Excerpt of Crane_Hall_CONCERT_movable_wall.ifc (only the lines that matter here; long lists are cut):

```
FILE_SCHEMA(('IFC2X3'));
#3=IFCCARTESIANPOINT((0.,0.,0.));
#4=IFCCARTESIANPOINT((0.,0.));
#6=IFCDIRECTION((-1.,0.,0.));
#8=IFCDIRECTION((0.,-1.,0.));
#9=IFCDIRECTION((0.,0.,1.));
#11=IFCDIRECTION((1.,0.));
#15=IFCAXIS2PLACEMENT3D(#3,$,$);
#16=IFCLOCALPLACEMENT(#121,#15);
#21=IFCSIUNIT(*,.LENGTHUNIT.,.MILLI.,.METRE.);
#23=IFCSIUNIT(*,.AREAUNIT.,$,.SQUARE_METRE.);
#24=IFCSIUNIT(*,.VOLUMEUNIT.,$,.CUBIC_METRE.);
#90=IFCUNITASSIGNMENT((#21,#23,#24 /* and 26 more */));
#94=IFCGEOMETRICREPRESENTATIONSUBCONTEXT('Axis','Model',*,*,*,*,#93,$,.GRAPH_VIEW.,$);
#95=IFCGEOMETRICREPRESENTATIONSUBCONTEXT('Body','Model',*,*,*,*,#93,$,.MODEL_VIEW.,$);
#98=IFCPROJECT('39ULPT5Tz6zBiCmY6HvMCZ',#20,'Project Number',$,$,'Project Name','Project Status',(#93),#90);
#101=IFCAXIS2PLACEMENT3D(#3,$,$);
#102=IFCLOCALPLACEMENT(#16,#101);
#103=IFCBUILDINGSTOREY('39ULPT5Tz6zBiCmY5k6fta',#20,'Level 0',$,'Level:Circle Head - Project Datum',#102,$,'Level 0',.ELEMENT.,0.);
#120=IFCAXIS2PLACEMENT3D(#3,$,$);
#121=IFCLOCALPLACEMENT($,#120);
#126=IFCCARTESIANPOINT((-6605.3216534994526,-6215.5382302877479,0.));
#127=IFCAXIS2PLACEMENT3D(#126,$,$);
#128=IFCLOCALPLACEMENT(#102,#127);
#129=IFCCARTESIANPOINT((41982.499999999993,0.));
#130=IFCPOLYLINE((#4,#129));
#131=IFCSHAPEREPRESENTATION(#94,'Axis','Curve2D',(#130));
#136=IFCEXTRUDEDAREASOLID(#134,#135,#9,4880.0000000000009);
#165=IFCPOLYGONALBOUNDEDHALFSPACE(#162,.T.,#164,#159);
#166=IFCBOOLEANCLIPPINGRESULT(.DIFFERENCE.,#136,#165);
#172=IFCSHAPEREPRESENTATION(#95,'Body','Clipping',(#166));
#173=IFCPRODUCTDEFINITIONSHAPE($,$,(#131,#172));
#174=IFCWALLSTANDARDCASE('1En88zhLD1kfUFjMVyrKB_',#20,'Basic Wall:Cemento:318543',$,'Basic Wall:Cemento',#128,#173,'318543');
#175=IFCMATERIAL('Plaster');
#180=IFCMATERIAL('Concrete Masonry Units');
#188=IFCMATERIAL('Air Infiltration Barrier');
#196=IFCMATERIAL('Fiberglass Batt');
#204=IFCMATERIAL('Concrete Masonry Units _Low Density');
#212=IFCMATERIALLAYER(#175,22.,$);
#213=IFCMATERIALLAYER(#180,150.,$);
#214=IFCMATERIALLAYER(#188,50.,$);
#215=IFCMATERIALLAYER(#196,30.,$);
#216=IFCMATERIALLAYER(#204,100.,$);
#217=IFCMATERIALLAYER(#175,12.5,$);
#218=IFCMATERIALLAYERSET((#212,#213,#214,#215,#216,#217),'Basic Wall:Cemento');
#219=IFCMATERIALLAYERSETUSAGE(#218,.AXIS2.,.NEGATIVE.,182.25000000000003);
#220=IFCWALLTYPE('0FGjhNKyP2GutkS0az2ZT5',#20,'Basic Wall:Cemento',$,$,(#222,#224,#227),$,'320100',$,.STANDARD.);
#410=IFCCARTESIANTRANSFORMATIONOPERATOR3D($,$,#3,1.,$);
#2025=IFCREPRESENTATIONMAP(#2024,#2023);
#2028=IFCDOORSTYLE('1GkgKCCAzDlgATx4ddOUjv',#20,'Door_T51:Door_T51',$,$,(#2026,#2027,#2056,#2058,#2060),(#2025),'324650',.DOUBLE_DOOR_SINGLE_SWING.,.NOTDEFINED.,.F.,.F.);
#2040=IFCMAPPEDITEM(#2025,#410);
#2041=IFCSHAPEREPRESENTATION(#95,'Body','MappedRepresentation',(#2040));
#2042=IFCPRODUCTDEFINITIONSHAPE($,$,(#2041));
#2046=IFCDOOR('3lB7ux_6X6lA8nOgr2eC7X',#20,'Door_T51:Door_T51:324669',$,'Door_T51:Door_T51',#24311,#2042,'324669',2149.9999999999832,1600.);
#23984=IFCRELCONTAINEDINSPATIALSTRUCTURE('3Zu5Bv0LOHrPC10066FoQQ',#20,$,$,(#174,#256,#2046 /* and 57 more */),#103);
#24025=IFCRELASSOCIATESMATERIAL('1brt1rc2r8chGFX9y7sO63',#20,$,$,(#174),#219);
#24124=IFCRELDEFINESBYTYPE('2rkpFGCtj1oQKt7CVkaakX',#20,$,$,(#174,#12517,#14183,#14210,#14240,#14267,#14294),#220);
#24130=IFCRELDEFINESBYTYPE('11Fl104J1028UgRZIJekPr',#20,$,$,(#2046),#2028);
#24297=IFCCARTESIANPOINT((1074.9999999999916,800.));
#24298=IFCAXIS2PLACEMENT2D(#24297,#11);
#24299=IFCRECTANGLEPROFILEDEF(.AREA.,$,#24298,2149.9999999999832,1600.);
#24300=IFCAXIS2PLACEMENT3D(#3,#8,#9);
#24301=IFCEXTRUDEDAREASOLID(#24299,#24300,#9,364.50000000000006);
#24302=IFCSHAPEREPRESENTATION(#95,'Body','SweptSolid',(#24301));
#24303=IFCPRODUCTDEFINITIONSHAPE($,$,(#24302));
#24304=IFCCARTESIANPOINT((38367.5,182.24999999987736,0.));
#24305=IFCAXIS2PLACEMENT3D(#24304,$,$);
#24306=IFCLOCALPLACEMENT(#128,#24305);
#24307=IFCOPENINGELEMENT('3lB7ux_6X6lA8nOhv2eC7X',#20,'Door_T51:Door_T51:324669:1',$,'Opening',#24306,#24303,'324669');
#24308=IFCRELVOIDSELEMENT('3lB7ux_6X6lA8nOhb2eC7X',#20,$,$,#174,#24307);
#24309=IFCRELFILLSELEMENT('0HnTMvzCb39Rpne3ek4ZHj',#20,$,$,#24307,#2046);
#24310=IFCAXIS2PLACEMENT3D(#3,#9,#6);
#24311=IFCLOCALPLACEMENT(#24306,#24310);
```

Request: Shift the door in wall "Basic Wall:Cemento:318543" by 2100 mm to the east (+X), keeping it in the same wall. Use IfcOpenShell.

```python
import ifcopenshell
import ifcopenshell.api.geometry
import ifcopenshell.util.placement

model = ifcopenshell.open("Crane_Hall_CONCERT_movable_wall.ifc")

door = model.by_guid("3lB7ux_6X6lA8nOgr2eC7X")
opening = door.FillsVoids[0].RelatingOpeningElement
wall = opening.VoidsElements[0].RelatingBuildingElement

wall_matrix = ifcopenshell.util.placement.get_local_placement(wall.ObjectPlacement)
shift = wall_matrix[:3, 0] * 2100.0
before = ifcopenshell.util.placement.get_local_placement(door.ObjectPlacement)[:3, 3].copy()

# The door is placed relative to its opening, so it follows when the opening moves.
matrix = ifcopenshell.util.placement.get_local_placement(opening.ObjectPlacement)
matrix[:3, 3] += shift
ifcopenshell.api.geometry.edit_object_placement(
    model, product=opening, matrix=matrix, is_si=False, should_transform_children=True
)

after = ifcopenshell.util.placement.get_local_placement(door.ObjectPlacement)[:3, 3]
print("door moved by", (after - before).round(3) + 0.0)

model.write("Crane_Hall_CONCERT_movable_wall_v2.ifc")
```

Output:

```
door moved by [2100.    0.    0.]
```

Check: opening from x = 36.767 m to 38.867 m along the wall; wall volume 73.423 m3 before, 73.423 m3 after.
